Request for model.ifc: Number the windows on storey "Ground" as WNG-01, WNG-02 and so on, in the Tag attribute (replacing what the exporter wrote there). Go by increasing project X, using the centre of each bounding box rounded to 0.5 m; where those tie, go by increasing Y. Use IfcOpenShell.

First a look at what the model holds.

```python
import ifcopenshell
import ifcopenshell.util.element
import ifcopenshell.util.placement

model = ifcopenshell.open("model.ifc")
print(model.schema)
storey = next(s for s in model.by_type("IfcBuildingStorey") if s.Name == "Ground")
windows = [e for e in ifcopenshell.util.element.get_decomposition(storey) if e.is_a("IfcWindow")]
for e in sorted(windows, key=lambda e: e.id()):
    origin = ifcopenshell.util.placement.get_local_placement(e.ObjectPlacement)[:3, 3]
    print(e.id(), e.Tag, e.Name, origin.round(2) + 0.0, sep=" | ")
```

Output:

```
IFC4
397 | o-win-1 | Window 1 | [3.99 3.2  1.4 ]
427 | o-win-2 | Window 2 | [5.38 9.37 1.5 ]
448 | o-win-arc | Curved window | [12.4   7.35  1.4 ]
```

```python
import ifcopenshell
import ifcopenshell.geom
import ifcopenshell.util.element
import ifcopenshell.util.shape

model = ifcopenshell.open("model.ifc")
settings = ifcopenshell.geom.settings()
settings.set("use-world-coords", True)


def centre(element):
    shape = ifcopenshell.geom.create_shape(settings, element)
    return ifcopenshell.util.shape.get_bbox_centroid(shape.geometry)


storey = next(s for s in model.by_type("IfcBuildingStorey") if s.Name == "Ground")
windows = [e for e in ifcopenshell.util.element.get_decomposition(storey) if e.is_a("IfcWindow")]

# Insertion points can sit at a corner or the storey origin, so sort by the geometry (in metres).
centres = {e: centre(e) for e in windows}
windows.sort(key=lambda e: (round(centres[e][0] / 0.5), centres[e][1]))

for i, e in enumerate(windows, start=1):
    number = f"WNG-{i:02d}"
    e.Tag = number
    print(e.id(), number)

model.write("model_rev.ifc")
```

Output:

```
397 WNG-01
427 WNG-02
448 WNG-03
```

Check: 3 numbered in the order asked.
